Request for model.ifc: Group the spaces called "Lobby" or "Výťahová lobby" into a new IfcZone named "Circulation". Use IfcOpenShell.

First a look at what the model holds.

```python
import ifcopenshell

model = ifcopenshell.open("model.ifc")
print(model.schema)
seen = {}
for space in model.by_type("IfcSpace"):
    seen[space.LongName] = seen.get(space.LongName, 0) + 1
for name, count in sorted(seen.items(), key=str):
    print(count, "x", name)
print("zones:", [z.Name for z in model.by_type("IfcZone")][:20])
```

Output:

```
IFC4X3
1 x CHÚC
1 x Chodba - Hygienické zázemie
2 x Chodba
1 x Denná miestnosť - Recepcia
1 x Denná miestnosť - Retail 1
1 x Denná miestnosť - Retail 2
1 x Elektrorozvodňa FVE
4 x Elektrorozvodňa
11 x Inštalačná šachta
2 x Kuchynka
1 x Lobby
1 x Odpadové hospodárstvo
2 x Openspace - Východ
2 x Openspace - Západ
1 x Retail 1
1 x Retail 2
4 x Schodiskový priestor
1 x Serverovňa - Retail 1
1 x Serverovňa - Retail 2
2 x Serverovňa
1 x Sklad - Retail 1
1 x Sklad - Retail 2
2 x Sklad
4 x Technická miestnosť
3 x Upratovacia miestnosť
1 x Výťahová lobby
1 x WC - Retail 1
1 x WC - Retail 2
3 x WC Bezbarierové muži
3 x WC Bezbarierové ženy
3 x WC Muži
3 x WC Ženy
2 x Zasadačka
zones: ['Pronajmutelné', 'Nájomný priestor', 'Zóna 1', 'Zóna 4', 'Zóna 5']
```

```python
import ifcopenshell
import ifcopenshell.api.group
import ifcopenshell.api.root

model = ifcopenshell.open("model.ifc")

names = {"Lobby", "Výťahová lobby"}
spaces = [s for s in model.by_type("IfcSpace") if s.LongName in names]

zone = ifcopenshell.api.root.create_entity(model, ifc_class="IfcZone", name="Circulation")
ifcopenshell.api.group.assign_group(model, products=spaces, group=zone)
print(len(spaces), "spaces in", zone.Name)

model.write("model_updated.ifc")
```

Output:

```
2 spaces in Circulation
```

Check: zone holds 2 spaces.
